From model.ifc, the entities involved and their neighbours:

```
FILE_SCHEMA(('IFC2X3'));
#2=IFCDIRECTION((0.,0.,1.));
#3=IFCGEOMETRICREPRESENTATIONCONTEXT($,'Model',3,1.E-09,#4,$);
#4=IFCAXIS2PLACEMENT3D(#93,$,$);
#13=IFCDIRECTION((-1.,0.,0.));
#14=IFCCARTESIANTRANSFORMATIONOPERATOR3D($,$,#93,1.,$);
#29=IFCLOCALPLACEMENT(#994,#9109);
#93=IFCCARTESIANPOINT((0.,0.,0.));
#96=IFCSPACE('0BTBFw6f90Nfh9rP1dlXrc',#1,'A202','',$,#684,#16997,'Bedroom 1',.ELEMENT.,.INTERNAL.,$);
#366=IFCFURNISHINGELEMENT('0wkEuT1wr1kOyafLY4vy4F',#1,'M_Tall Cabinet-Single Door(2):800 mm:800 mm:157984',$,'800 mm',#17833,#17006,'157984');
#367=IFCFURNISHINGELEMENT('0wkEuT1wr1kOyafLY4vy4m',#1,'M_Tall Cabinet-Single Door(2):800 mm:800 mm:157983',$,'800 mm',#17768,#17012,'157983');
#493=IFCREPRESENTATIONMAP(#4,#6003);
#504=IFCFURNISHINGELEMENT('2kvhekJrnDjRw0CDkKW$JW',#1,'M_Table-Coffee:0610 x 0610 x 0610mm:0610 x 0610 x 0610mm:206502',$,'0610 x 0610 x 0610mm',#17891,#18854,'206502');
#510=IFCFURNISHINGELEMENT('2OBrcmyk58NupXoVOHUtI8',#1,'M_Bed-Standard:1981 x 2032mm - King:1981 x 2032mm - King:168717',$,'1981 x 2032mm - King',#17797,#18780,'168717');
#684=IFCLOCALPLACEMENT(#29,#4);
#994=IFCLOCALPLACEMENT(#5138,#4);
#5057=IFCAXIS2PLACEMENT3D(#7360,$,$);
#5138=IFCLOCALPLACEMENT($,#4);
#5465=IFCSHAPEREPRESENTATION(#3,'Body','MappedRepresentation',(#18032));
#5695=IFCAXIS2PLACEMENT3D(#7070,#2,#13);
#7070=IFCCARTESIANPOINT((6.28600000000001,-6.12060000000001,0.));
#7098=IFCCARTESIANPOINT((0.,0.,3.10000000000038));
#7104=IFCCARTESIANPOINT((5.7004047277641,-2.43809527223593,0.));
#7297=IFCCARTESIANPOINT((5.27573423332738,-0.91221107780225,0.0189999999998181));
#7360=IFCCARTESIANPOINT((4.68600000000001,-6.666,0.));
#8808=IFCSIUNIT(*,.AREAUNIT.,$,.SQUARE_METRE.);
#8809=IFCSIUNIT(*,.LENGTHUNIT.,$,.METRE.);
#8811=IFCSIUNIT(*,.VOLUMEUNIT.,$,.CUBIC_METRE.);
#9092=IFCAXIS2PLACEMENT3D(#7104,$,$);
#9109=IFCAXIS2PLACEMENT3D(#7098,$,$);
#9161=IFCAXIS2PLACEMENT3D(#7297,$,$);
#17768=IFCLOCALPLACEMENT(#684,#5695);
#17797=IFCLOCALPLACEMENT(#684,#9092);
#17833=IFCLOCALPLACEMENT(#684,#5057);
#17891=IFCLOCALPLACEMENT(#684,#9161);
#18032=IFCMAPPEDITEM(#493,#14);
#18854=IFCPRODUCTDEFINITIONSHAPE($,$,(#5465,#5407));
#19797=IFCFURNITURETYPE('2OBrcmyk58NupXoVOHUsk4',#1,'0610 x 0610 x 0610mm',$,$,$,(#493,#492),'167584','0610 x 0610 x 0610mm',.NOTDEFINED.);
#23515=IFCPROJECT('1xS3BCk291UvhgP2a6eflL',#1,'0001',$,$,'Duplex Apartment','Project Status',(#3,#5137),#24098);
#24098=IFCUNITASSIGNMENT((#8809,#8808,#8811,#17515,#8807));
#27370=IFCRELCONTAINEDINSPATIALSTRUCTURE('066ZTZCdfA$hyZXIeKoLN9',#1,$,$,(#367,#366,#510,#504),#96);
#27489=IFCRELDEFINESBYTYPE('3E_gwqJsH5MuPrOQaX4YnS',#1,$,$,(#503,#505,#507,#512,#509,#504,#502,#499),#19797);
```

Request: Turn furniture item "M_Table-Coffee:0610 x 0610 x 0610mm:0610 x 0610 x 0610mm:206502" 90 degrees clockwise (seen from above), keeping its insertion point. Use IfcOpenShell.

```python
import ifcopenshell
import ifcopenshell.api.geometry
import ifcopenshell.util.placement

model = ifcopenshell.open("model.ifc")

item = model.by_guid("2kvhekJrnDjRw0CDkKW$JW")
matrix = ifcopenshell.util.placement.get_local_placement(item.ObjectPlacement)
matrix = matrix @ ifcopenshell.util.placement.rotation(-90, "Z")
ifcopenshell.api.geometry.edit_object_placement(model, product=item, matrix=matrix, is_si=False)

print(ifcopenshell.util.placement.get_local_placement(item.ObjectPlacement).round(3) + 0.0)

model.write("model_updated.ifc")
```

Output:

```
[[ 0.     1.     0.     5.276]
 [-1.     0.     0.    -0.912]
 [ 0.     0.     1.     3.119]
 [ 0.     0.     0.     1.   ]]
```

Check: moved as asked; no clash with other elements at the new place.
